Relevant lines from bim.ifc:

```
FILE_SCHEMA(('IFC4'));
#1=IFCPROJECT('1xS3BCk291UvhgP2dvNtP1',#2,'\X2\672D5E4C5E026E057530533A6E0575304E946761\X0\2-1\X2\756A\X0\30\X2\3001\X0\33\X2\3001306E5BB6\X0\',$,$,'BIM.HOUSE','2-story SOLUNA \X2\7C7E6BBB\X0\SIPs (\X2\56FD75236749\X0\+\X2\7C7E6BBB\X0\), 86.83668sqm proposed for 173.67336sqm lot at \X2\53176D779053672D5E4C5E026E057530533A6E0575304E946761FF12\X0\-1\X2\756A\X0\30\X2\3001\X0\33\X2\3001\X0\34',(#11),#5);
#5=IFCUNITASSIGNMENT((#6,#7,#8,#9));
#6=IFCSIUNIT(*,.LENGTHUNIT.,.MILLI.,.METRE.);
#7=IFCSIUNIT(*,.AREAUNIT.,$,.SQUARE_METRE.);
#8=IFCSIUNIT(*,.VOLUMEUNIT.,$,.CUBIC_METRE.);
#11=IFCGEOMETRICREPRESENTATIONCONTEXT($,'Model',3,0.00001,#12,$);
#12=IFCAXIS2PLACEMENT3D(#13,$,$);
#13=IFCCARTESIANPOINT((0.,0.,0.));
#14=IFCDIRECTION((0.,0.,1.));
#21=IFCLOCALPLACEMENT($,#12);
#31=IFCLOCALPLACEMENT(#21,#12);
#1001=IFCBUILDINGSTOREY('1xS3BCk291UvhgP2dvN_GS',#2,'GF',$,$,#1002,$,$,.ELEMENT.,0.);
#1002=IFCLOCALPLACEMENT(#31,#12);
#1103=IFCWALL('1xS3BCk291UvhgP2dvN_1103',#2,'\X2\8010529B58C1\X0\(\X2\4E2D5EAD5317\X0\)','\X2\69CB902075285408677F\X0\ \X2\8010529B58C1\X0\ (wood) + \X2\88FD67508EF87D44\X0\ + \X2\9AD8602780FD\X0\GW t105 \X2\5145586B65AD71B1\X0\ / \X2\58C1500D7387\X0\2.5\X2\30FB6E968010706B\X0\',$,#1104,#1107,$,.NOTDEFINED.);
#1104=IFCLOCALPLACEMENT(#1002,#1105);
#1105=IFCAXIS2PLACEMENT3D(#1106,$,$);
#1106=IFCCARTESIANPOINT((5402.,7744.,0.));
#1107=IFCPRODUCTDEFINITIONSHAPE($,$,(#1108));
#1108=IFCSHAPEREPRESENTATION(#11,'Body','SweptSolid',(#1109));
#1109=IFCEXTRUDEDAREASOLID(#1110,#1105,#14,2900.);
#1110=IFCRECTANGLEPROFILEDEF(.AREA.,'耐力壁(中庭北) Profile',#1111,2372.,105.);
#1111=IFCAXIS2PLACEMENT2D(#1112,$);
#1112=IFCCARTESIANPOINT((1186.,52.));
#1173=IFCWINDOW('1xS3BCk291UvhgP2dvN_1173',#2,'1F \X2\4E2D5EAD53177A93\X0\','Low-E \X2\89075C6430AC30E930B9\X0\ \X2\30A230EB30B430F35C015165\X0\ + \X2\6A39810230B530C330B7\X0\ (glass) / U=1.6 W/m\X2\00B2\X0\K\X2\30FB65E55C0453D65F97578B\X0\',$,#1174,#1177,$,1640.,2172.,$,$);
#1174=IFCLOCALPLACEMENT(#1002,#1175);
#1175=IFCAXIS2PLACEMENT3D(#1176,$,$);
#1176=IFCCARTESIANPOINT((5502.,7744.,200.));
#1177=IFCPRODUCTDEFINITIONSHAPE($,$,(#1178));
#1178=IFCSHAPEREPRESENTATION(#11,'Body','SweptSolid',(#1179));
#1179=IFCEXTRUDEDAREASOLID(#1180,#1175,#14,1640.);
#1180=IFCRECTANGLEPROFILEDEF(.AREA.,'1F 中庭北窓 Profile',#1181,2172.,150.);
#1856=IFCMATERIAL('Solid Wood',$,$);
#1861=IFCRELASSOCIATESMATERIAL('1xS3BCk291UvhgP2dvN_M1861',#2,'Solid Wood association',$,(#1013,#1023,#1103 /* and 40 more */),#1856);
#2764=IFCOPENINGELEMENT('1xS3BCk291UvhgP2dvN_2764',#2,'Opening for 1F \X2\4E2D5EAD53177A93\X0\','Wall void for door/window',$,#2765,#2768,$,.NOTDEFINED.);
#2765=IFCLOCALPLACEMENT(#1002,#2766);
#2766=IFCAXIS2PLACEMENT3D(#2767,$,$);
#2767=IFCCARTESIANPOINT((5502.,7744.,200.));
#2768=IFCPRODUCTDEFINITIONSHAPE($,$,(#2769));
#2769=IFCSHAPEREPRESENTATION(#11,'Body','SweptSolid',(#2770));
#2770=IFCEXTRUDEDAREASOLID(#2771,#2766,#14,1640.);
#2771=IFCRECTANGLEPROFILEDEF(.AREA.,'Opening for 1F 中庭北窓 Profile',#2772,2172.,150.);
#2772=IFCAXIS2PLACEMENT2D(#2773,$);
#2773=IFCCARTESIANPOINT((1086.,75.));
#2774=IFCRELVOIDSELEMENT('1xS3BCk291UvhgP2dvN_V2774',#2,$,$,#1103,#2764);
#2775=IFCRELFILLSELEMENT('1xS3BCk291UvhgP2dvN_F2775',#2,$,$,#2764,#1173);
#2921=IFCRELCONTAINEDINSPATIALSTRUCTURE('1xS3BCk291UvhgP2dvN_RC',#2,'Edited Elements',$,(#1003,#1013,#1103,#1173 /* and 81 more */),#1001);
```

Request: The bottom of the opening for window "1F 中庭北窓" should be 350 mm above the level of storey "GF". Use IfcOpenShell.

```python
import numpy as np
import ifcopenshell
import ifcopenshell.api.geometry
import ifcopenshell.geom
import ifcopenshell.util.element
import ifcopenshell.util.placement
import ifcopenshell.util.shape
import ifcopenshell.util.unit

model = ifcopenshell.open("bim.ifc")
unit_scale = ifcopenshell.util.unit.calculate_unit_scale(model)

window = model.by_id(1173)
opening = window.FillsVoids[0].RelatingOpeningElement
storey = ifcopenshell.util.element.get_container(window, ifc_class="IfcBuildingStorey")
level = ifcopenshell.util.placement.get_local_placement(storey.ObjectPlacement)[2, 3]

# The opening's origin need not be at the sill, so measure its lowest point.
shape = ifcopenshell.geom.create_shape(ifcopenshell.geom.settings(), opening)
bottom = ifcopenshell.util.shape.get_shape_bottom_elevation(shape, shape.geometry) / unit_scale
dz = level + 0.35 / unit_scale - bottom

shift = np.array([0.0, 0.0, dz])
# The window is not placed relative to its opening, so move both.
for product in (opening, window):
    matrix = ifcopenshell.util.placement.get_local_placement(product.ObjectPlacement)
    matrix[:3, 3] += shift
    ifcopenshell.api.geometry.edit_object_placement(model, product=product, matrix=matrix, is_si=False)

print(f"moved by {dz * unit_scale:+.3f} m")

model.write("bim-out.ifc")
```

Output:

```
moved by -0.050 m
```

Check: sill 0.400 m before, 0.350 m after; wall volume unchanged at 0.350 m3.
